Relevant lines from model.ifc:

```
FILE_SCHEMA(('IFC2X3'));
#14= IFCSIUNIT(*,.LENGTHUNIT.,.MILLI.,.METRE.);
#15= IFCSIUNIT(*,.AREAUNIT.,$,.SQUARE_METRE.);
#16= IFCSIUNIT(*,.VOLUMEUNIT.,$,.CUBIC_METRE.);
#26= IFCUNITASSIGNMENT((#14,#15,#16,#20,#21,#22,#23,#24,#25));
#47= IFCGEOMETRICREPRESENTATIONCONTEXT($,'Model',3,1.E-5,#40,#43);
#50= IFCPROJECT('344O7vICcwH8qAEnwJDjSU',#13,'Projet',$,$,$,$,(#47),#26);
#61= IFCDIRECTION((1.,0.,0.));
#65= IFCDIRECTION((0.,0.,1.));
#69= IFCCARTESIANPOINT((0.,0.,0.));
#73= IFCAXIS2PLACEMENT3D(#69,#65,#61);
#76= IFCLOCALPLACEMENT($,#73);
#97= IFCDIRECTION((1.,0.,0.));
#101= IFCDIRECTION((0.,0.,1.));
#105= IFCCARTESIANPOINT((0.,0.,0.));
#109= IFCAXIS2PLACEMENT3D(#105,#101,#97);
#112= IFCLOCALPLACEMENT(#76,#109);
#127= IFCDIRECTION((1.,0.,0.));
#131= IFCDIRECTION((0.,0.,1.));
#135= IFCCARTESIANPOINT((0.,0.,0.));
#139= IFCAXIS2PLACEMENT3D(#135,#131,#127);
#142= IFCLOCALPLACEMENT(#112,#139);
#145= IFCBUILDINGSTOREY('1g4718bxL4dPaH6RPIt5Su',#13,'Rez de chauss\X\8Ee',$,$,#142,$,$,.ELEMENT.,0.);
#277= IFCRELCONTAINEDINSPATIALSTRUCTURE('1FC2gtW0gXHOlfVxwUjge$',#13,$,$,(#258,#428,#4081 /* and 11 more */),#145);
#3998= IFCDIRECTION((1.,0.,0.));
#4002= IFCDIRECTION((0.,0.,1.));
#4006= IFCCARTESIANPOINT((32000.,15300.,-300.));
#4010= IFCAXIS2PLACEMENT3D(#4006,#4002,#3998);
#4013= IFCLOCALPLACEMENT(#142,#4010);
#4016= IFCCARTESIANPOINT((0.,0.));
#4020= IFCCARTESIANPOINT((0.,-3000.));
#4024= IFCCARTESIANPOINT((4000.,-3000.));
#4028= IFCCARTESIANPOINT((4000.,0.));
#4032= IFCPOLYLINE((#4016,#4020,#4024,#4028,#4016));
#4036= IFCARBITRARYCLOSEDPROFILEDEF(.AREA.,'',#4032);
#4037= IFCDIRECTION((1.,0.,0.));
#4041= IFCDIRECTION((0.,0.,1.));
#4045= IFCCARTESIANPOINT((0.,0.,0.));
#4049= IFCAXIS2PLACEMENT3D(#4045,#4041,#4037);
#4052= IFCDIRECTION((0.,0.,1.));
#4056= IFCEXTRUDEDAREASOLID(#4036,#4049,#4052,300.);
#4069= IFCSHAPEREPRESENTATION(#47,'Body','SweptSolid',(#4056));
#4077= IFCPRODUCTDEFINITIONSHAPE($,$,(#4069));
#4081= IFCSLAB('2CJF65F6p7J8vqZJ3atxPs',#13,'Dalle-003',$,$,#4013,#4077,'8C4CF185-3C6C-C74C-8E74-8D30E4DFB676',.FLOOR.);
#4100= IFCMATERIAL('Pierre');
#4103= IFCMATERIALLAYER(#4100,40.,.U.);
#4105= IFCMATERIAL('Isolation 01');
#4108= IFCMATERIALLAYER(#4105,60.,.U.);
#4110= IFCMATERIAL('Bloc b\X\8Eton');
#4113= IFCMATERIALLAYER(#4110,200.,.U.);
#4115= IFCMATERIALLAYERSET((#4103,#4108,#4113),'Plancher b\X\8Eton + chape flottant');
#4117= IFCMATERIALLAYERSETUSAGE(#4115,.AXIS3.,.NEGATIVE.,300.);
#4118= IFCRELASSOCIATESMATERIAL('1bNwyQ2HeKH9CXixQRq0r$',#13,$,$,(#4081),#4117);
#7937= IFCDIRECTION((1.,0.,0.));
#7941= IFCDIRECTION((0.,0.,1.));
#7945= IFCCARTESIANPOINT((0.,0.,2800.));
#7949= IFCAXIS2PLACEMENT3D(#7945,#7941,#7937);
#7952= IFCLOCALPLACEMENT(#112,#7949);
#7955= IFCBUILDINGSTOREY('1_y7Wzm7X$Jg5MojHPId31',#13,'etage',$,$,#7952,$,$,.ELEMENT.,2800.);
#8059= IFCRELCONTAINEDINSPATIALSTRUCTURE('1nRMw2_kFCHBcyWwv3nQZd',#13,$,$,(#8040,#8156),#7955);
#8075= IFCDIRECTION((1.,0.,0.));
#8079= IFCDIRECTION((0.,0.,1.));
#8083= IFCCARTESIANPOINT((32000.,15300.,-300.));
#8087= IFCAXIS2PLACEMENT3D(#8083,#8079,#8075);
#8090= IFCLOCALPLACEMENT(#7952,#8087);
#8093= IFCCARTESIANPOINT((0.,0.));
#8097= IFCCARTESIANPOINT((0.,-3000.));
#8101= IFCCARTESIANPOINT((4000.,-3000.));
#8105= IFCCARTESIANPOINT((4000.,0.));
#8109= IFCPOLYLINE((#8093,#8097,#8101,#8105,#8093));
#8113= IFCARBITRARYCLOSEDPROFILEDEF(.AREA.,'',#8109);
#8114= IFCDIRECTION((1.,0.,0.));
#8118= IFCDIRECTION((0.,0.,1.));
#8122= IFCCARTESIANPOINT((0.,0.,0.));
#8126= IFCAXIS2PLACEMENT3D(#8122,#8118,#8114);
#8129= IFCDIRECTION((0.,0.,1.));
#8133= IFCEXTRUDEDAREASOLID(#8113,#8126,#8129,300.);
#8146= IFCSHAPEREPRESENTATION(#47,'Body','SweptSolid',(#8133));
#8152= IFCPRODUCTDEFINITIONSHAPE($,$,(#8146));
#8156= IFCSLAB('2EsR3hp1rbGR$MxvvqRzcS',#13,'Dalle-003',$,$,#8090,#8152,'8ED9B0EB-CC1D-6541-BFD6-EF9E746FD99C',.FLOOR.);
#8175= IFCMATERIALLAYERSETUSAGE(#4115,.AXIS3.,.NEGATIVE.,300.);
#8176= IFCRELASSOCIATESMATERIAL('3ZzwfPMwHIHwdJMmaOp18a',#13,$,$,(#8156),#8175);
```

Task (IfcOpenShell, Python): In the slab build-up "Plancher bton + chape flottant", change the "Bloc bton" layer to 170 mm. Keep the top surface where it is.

```python
import ifcopenshell
import ifcopenshell.util.element
import ifcopenshell.util.unit

model = ifcopenshell.open("model.ifc")
unit_scale = ifcopenshell.util.unit.calculate_unit_scale(model)

layer_set = model.by_id(4115)
layer = next(l for l in layer_set.MaterialLayers if l.Material and l.Material.Name == 'Bloc b\x8eton')
change = 0.17 / unit_scale - layer.LayerThickness
layer.LayerThickness += change

# The layer set is shared, so every slab that uses it gets the new thickness.
slabs = [e for e in ifcopenshell.util.element.get_elements_by_material(model, layer_set) if e.is_a("IfcSlab")]
for slab in sorted(slabs, key=lambda e: e.id()):
    body = next(r for r in slab.Representation.Representations if r.RepresentationIdentifier == "Body")
    solid = body.Items[0]
    old_depth = solid.Depth
    solid.Depth += change
    # Extruded upwards: lower the start of the extrusion so the top stays.
    x, y, z = solid.Position.Location.Coordinates
    solid.Position.Location = model.createIfcCartesianPoint((x, y, z - change))
    print(slab.id(), f"{old_depth:g} -> {solid.Depth:g}")

model.write("model_rev.ifc")
```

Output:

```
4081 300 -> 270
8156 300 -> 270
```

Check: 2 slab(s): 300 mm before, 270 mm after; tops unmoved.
